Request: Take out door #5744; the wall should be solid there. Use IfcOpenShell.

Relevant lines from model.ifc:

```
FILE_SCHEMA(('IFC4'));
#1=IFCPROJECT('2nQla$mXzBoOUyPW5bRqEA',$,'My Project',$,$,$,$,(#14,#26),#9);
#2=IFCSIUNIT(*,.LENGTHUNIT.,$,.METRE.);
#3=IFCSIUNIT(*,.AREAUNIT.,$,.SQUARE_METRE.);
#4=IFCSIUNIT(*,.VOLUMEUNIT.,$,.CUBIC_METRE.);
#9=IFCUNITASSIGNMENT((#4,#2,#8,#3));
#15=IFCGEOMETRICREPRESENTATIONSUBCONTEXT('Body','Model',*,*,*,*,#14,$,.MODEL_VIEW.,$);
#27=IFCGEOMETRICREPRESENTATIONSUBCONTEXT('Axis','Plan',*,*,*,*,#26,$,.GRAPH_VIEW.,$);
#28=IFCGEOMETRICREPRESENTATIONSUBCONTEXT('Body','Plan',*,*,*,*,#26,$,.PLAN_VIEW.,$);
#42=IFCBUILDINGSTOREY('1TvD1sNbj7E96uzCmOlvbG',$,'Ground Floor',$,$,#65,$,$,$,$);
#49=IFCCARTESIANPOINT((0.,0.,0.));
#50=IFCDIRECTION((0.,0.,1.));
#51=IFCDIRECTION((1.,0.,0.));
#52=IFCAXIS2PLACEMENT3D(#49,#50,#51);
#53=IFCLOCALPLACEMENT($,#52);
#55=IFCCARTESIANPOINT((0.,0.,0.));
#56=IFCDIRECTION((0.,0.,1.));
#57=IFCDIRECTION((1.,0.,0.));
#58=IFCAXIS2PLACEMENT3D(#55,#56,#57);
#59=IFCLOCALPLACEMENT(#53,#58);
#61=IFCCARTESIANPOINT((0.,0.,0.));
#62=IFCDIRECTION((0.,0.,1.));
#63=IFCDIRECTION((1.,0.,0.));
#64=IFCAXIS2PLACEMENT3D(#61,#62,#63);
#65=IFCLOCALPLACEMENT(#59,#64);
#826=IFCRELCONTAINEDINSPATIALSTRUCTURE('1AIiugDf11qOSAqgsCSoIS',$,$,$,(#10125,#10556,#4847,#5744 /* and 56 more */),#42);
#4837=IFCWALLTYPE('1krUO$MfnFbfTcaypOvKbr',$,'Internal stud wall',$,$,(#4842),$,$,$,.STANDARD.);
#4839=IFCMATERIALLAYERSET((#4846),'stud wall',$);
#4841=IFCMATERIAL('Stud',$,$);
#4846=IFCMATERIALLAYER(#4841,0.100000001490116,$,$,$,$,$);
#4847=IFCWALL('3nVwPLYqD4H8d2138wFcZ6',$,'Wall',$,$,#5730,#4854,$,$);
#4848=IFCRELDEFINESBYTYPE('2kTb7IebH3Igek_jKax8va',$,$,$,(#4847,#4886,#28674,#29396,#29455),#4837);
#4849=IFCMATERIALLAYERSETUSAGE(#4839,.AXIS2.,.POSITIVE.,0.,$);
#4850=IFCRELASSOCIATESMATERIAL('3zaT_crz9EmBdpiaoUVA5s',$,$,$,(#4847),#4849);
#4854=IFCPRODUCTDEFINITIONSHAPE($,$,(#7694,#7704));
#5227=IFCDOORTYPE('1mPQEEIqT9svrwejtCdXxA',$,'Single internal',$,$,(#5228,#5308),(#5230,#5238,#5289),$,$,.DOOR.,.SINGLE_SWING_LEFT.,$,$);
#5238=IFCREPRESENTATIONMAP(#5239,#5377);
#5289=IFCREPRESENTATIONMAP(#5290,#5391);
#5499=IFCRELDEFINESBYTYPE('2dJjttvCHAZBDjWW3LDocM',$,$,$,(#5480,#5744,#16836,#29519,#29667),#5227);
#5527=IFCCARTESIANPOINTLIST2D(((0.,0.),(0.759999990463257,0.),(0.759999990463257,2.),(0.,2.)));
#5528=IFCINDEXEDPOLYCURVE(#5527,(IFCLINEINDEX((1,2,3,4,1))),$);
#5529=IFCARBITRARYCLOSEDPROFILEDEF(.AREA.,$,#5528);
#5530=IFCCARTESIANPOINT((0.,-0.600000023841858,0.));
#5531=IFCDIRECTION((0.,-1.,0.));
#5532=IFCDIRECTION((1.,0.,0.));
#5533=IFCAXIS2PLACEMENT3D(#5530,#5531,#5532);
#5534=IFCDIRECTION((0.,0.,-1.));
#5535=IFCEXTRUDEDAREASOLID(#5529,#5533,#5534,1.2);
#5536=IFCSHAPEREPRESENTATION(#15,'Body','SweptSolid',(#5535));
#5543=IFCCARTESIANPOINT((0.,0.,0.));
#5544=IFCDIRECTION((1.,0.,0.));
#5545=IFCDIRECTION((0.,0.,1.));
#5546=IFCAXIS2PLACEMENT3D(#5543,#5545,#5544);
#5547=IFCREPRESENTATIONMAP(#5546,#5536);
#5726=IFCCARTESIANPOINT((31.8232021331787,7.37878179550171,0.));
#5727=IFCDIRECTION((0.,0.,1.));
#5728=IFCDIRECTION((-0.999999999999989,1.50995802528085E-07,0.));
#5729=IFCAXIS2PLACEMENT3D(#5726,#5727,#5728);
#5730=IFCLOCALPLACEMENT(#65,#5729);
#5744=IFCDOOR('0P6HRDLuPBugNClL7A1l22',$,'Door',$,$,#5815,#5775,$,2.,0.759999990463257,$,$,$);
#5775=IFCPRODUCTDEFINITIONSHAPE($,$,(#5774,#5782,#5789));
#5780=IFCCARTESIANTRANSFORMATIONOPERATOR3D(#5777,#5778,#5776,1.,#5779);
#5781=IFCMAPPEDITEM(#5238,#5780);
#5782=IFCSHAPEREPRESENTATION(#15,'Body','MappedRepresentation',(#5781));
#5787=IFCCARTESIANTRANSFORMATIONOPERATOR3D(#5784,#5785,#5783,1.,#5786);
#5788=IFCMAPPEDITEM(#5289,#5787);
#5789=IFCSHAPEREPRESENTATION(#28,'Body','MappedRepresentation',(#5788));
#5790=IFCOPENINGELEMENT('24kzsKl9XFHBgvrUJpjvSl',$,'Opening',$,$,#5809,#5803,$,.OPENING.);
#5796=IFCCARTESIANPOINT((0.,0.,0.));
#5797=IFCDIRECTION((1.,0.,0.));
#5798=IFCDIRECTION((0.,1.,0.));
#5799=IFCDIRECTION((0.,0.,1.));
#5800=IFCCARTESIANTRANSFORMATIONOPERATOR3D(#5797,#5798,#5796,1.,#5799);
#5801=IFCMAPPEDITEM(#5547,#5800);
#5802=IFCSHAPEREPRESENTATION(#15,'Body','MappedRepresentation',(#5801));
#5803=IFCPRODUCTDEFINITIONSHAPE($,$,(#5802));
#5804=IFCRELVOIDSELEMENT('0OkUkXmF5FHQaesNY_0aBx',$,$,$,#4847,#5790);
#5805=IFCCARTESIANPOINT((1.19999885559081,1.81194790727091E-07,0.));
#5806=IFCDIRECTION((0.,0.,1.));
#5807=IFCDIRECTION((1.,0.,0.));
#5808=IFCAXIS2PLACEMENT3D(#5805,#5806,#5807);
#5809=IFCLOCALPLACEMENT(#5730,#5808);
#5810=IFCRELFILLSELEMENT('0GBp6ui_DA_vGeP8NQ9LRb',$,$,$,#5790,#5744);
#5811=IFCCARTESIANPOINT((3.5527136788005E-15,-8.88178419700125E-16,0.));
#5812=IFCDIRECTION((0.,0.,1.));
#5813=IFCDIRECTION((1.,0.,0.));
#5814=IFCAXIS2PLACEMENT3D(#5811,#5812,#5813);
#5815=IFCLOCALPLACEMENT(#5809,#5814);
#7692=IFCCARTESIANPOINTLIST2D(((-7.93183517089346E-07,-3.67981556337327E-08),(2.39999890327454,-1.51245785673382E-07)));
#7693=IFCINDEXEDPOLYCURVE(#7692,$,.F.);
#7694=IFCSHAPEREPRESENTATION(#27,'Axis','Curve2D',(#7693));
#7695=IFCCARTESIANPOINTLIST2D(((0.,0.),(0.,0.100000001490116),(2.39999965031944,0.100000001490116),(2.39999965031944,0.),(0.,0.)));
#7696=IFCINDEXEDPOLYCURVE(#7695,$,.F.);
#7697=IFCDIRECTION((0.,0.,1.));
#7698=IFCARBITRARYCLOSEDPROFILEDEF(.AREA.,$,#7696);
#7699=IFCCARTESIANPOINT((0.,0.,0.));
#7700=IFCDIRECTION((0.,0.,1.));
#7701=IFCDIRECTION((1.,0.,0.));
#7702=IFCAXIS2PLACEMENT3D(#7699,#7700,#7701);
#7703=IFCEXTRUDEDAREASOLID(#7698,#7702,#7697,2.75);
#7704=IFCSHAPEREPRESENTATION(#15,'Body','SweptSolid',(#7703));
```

```python
import ifcopenshell
import ifcopenshell.api.feature
import ifcopenshell.api.root
import ifcopenshell.geom
import ifcopenshell.util.shape

model = ifcopenshell.open("model.ifc")
settings = ifcopenshell.geom.settings()


def volume(element):
    """Net volume in cubic metres, openings subtracted."""
    shape = ifcopenshell.geom.create_shape(settings, element)
    return ifcopenshell.util.shape.get_volume(shape.geometry)


door = model.by_guid("0P6HRDLuPBugNClL7A1l22")
opening = door.FillsVoids[0].RelatingOpeningElement
wall = opening.VoidsElements[0].RelatingBuildingElement
before = volume(wall)

ifcopenshell.api.root.remove_product(model, product=door)
ifcopenshell.api.feature.remove_feature(model, feature=opening)

after = volume(wall)

print(f"wall volume {before:.3f} -> {after:.3f} m3")

model.write("model_v2.ifc")
```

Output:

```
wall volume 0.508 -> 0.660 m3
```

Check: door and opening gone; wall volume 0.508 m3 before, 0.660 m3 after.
